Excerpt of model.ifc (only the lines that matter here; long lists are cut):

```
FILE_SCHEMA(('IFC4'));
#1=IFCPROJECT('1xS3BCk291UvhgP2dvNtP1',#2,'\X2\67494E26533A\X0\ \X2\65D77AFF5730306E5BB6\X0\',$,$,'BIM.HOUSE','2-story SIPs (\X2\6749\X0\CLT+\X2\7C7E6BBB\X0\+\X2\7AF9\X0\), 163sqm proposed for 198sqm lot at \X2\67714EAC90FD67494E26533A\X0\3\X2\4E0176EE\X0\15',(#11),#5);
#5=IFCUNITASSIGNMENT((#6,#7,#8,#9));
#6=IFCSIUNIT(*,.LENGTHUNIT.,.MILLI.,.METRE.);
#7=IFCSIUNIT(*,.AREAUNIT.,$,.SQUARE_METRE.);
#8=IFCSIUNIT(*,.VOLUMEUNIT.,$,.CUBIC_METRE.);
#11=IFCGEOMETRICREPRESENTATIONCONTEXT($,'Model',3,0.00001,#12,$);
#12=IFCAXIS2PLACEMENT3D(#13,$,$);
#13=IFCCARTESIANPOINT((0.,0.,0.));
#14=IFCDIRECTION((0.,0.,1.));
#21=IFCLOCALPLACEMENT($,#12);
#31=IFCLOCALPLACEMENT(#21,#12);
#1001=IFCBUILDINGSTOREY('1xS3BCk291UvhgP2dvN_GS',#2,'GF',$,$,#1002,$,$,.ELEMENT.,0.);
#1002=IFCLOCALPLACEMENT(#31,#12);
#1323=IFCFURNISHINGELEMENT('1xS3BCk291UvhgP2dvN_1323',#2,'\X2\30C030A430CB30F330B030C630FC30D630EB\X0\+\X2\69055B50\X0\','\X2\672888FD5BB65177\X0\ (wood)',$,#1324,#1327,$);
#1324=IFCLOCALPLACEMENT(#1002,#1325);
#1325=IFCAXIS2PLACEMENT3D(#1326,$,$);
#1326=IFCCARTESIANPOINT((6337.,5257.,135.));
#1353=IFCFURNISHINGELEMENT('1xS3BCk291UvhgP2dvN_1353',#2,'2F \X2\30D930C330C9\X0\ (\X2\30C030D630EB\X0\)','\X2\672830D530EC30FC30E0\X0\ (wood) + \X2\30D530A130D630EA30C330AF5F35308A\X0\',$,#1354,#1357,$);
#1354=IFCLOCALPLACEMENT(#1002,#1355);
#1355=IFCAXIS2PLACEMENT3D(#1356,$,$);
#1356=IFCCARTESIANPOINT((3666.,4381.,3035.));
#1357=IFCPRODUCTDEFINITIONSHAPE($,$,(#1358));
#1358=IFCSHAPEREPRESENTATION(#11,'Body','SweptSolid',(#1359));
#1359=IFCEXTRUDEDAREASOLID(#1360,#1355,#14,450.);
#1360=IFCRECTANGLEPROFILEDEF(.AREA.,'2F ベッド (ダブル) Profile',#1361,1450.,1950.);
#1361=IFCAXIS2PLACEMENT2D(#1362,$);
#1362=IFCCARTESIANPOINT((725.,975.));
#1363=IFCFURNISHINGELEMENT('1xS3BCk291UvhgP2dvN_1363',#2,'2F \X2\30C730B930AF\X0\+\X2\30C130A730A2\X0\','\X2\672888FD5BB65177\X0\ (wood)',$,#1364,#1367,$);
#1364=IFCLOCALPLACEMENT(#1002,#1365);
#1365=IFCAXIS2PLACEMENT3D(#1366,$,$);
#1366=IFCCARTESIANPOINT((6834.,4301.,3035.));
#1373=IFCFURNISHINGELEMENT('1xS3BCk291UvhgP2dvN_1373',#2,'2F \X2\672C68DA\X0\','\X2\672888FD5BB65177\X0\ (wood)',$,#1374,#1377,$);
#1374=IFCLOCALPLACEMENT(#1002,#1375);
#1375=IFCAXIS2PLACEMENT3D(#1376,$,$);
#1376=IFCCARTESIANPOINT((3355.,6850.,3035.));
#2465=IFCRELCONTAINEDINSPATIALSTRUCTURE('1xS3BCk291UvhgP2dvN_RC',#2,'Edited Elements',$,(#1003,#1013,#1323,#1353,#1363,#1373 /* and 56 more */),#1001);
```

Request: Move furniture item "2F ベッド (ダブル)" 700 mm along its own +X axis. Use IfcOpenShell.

```python
import ifcopenshell
import ifcopenshell.api.geometry
import ifcopenshell.util.placement
import ifcopenshell.util.unit

model = ifcopenshell.open("model.ifc")
unit_scale = ifcopenshell.util.unit.calculate_unit_scale(model)

item = model.by_id(1353)
matrix = ifcopenshell.util.placement.get_local_placement(item.ObjectPlacement)
matrix[:3, 3] += matrix[:3, 0] * 0.7 / unit_scale
ifcopenshell.api.geometry.edit_object_placement(model, product=item, matrix=matrix, is_si=False)

print(ifcopenshell.util.placement.get_local_placement(item.ObjectPlacement).round(3) + 0.0)

model.write("model_updated.ifc")
```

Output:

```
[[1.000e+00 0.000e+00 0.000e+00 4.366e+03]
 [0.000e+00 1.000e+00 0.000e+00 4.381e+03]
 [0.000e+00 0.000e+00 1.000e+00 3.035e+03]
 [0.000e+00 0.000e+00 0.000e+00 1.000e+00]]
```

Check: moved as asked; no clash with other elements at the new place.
